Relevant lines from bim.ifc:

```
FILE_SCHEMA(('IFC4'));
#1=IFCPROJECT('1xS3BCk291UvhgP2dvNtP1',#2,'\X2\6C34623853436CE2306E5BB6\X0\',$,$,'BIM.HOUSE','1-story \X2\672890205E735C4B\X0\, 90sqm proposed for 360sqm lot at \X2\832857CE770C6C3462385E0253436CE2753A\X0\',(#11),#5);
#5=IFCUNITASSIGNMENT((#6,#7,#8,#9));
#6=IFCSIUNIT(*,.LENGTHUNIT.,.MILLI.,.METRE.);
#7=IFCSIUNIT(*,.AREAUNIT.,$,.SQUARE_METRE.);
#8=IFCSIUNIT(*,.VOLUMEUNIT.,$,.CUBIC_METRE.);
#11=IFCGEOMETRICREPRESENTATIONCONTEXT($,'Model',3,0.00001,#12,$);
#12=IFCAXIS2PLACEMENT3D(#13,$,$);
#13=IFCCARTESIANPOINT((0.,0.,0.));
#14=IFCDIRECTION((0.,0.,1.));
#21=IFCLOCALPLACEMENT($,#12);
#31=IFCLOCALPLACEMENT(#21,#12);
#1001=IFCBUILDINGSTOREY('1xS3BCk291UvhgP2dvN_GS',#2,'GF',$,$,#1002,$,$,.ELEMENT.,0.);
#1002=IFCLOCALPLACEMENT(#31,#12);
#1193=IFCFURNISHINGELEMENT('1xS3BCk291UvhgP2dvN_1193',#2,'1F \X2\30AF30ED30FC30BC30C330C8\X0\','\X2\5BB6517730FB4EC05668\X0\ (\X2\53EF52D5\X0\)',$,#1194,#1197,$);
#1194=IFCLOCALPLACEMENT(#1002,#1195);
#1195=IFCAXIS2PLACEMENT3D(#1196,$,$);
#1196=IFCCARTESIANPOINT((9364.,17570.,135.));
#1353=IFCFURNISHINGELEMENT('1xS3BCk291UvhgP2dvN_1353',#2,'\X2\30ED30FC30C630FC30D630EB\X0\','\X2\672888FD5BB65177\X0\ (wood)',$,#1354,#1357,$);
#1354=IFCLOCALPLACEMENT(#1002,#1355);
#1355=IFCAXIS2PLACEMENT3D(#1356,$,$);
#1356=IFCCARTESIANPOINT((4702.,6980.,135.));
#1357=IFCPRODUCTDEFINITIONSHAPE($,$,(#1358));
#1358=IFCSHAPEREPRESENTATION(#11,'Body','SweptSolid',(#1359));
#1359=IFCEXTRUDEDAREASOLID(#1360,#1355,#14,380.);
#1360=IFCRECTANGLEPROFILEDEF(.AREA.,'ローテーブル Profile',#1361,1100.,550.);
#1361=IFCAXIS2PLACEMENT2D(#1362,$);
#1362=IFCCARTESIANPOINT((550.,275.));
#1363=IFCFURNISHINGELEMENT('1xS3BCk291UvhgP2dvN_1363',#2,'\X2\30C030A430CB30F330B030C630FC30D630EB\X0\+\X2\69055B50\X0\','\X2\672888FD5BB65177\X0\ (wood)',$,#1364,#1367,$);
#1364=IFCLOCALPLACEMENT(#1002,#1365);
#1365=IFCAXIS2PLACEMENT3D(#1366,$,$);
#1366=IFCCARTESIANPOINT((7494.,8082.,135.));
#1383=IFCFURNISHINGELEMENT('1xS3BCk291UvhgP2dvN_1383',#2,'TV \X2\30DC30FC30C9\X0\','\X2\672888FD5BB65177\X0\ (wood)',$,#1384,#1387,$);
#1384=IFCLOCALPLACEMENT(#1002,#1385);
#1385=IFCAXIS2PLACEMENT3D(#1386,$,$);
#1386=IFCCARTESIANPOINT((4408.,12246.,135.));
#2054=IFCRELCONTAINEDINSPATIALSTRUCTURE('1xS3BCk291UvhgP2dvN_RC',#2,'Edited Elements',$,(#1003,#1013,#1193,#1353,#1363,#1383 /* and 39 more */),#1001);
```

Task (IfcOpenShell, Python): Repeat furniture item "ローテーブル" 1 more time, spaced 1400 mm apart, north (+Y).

```python
import numpy as np
import ifcopenshell
import ifcopenshell.api.geometry
import ifcopenshell.api.root
import ifcopenshell.util.element
import ifcopenshell.util.placement
import ifcopenshell.util.unit

model = ifcopenshell.open("bim.ifc")
unit_scale = ifcopenshell.util.unit.calculate_unit_scale(model)


def reuse_history(source, copy):
    """copy_class also copies each property set's owner history, people and application; keep the originals."""
    for rel in copy.IsDefinedBy:
        if rel.is_a("IfcRelDefinesByProperties") and (history := rel.RelatingPropertyDefinition.OwnerHistory):
            rel.RelatingPropertyDefinition.OwnerHistory = source.OwnerHistory
            ifcopenshell.util.element.remove_deep2(model, history)


source = model.by_guid("1xS3BCk291UvhgP2dvN_1353")
base = ifcopenshell.util.placement.get_local_placement(source.ObjectPlacement)
step = np.array([0.0, 1.0, 0.0]) * 1.4 / unit_scale

for i in range(1, 2):
    copy = ifcopenshell.api.root.copy_class(model, product=source)
    copy.Representation = ifcopenshell.util.element.copy_deep(
        model, source.Representation, exclude=["IfcGeometricRepresentationContext", "IfcRepresentationMap"]
    )
    reuse_history(source, copy)
    matrix = base.copy()
    matrix[:3, 3] += i * step
    print("added at", matrix[:3, 3].round(3) + 0.0)
    ifcopenshell.api.geometry.edit_object_placement(model, product=copy, matrix=matrix, is_si=False)

model.write("bim_edited.ifc")
```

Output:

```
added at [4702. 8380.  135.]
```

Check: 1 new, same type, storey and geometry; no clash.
